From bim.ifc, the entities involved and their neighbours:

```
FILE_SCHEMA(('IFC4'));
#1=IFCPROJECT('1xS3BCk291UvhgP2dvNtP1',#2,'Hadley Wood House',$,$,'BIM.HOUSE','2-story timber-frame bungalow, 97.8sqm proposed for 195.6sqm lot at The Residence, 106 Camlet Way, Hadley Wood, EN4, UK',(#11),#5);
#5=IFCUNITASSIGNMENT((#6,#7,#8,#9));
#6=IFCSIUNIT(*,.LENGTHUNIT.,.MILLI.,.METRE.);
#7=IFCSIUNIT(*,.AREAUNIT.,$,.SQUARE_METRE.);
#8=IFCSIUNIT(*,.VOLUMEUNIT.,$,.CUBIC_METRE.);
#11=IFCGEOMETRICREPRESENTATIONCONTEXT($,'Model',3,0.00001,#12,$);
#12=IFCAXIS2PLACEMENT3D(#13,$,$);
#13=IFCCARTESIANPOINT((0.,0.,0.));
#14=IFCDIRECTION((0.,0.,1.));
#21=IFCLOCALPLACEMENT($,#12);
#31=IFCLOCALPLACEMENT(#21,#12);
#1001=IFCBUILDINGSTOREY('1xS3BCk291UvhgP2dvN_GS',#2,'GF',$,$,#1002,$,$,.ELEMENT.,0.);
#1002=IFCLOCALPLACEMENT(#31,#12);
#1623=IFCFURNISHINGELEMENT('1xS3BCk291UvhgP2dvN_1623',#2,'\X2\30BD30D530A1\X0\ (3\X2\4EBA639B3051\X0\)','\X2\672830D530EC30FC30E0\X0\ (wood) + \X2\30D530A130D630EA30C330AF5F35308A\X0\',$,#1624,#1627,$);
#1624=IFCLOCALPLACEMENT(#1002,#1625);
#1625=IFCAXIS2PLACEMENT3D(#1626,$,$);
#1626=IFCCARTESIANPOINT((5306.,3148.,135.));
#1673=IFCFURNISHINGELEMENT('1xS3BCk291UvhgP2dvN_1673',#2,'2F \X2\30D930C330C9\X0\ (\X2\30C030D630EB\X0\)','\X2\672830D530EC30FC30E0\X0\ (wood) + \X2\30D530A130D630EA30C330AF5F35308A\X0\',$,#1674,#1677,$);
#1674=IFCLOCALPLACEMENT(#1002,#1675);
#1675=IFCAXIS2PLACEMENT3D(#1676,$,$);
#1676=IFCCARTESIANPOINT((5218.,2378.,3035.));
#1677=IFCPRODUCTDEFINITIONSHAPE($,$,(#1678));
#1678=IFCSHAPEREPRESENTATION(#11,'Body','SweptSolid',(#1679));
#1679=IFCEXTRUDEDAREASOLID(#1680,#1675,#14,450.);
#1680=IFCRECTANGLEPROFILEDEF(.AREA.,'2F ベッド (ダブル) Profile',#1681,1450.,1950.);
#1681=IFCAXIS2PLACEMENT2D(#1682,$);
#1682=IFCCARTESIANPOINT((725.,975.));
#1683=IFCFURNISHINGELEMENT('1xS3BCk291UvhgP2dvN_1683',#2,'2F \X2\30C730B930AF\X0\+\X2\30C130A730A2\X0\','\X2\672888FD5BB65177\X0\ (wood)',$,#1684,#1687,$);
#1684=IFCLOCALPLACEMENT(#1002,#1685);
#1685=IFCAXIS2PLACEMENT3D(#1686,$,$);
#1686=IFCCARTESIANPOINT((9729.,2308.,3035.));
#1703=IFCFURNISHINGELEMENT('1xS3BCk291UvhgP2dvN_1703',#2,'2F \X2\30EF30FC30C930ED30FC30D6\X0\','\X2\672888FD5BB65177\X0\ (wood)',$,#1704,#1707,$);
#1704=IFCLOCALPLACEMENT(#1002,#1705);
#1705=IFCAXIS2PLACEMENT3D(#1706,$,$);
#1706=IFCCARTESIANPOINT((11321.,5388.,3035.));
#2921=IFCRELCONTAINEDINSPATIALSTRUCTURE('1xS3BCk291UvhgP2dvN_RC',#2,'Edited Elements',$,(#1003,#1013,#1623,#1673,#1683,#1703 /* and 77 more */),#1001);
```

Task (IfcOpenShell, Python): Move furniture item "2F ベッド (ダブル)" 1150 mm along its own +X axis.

```python
import ifcopenshell
import ifcopenshell.api.geometry
import ifcopenshell.util.placement
import ifcopenshell.util.unit

model = ifcopenshell.open("bim.ifc")
unit_scale = ifcopenshell.util.unit.calculate_unit_scale(model)

item = model.by_guid("1xS3BCk291UvhgP2dvN_1673")
matrix = ifcopenshell.util.placement.get_local_placement(item.ObjectPlacement)
matrix[:3, 3] += matrix[:3, 0] * 1.15 / unit_scale
ifcopenshell.api.geometry.edit_object_placement(model, product=item, matrix=matrix, is_si=False)

print(ifcopenshell.util.placement.get_local_placement(item.ObjectPlacement).round(3) + 0.0)

model.write("bim-out.ifc")
```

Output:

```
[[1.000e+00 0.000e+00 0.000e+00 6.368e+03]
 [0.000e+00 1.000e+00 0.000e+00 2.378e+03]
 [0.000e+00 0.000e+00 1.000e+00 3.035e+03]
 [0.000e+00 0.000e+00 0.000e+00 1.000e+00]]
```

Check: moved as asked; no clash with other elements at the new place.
